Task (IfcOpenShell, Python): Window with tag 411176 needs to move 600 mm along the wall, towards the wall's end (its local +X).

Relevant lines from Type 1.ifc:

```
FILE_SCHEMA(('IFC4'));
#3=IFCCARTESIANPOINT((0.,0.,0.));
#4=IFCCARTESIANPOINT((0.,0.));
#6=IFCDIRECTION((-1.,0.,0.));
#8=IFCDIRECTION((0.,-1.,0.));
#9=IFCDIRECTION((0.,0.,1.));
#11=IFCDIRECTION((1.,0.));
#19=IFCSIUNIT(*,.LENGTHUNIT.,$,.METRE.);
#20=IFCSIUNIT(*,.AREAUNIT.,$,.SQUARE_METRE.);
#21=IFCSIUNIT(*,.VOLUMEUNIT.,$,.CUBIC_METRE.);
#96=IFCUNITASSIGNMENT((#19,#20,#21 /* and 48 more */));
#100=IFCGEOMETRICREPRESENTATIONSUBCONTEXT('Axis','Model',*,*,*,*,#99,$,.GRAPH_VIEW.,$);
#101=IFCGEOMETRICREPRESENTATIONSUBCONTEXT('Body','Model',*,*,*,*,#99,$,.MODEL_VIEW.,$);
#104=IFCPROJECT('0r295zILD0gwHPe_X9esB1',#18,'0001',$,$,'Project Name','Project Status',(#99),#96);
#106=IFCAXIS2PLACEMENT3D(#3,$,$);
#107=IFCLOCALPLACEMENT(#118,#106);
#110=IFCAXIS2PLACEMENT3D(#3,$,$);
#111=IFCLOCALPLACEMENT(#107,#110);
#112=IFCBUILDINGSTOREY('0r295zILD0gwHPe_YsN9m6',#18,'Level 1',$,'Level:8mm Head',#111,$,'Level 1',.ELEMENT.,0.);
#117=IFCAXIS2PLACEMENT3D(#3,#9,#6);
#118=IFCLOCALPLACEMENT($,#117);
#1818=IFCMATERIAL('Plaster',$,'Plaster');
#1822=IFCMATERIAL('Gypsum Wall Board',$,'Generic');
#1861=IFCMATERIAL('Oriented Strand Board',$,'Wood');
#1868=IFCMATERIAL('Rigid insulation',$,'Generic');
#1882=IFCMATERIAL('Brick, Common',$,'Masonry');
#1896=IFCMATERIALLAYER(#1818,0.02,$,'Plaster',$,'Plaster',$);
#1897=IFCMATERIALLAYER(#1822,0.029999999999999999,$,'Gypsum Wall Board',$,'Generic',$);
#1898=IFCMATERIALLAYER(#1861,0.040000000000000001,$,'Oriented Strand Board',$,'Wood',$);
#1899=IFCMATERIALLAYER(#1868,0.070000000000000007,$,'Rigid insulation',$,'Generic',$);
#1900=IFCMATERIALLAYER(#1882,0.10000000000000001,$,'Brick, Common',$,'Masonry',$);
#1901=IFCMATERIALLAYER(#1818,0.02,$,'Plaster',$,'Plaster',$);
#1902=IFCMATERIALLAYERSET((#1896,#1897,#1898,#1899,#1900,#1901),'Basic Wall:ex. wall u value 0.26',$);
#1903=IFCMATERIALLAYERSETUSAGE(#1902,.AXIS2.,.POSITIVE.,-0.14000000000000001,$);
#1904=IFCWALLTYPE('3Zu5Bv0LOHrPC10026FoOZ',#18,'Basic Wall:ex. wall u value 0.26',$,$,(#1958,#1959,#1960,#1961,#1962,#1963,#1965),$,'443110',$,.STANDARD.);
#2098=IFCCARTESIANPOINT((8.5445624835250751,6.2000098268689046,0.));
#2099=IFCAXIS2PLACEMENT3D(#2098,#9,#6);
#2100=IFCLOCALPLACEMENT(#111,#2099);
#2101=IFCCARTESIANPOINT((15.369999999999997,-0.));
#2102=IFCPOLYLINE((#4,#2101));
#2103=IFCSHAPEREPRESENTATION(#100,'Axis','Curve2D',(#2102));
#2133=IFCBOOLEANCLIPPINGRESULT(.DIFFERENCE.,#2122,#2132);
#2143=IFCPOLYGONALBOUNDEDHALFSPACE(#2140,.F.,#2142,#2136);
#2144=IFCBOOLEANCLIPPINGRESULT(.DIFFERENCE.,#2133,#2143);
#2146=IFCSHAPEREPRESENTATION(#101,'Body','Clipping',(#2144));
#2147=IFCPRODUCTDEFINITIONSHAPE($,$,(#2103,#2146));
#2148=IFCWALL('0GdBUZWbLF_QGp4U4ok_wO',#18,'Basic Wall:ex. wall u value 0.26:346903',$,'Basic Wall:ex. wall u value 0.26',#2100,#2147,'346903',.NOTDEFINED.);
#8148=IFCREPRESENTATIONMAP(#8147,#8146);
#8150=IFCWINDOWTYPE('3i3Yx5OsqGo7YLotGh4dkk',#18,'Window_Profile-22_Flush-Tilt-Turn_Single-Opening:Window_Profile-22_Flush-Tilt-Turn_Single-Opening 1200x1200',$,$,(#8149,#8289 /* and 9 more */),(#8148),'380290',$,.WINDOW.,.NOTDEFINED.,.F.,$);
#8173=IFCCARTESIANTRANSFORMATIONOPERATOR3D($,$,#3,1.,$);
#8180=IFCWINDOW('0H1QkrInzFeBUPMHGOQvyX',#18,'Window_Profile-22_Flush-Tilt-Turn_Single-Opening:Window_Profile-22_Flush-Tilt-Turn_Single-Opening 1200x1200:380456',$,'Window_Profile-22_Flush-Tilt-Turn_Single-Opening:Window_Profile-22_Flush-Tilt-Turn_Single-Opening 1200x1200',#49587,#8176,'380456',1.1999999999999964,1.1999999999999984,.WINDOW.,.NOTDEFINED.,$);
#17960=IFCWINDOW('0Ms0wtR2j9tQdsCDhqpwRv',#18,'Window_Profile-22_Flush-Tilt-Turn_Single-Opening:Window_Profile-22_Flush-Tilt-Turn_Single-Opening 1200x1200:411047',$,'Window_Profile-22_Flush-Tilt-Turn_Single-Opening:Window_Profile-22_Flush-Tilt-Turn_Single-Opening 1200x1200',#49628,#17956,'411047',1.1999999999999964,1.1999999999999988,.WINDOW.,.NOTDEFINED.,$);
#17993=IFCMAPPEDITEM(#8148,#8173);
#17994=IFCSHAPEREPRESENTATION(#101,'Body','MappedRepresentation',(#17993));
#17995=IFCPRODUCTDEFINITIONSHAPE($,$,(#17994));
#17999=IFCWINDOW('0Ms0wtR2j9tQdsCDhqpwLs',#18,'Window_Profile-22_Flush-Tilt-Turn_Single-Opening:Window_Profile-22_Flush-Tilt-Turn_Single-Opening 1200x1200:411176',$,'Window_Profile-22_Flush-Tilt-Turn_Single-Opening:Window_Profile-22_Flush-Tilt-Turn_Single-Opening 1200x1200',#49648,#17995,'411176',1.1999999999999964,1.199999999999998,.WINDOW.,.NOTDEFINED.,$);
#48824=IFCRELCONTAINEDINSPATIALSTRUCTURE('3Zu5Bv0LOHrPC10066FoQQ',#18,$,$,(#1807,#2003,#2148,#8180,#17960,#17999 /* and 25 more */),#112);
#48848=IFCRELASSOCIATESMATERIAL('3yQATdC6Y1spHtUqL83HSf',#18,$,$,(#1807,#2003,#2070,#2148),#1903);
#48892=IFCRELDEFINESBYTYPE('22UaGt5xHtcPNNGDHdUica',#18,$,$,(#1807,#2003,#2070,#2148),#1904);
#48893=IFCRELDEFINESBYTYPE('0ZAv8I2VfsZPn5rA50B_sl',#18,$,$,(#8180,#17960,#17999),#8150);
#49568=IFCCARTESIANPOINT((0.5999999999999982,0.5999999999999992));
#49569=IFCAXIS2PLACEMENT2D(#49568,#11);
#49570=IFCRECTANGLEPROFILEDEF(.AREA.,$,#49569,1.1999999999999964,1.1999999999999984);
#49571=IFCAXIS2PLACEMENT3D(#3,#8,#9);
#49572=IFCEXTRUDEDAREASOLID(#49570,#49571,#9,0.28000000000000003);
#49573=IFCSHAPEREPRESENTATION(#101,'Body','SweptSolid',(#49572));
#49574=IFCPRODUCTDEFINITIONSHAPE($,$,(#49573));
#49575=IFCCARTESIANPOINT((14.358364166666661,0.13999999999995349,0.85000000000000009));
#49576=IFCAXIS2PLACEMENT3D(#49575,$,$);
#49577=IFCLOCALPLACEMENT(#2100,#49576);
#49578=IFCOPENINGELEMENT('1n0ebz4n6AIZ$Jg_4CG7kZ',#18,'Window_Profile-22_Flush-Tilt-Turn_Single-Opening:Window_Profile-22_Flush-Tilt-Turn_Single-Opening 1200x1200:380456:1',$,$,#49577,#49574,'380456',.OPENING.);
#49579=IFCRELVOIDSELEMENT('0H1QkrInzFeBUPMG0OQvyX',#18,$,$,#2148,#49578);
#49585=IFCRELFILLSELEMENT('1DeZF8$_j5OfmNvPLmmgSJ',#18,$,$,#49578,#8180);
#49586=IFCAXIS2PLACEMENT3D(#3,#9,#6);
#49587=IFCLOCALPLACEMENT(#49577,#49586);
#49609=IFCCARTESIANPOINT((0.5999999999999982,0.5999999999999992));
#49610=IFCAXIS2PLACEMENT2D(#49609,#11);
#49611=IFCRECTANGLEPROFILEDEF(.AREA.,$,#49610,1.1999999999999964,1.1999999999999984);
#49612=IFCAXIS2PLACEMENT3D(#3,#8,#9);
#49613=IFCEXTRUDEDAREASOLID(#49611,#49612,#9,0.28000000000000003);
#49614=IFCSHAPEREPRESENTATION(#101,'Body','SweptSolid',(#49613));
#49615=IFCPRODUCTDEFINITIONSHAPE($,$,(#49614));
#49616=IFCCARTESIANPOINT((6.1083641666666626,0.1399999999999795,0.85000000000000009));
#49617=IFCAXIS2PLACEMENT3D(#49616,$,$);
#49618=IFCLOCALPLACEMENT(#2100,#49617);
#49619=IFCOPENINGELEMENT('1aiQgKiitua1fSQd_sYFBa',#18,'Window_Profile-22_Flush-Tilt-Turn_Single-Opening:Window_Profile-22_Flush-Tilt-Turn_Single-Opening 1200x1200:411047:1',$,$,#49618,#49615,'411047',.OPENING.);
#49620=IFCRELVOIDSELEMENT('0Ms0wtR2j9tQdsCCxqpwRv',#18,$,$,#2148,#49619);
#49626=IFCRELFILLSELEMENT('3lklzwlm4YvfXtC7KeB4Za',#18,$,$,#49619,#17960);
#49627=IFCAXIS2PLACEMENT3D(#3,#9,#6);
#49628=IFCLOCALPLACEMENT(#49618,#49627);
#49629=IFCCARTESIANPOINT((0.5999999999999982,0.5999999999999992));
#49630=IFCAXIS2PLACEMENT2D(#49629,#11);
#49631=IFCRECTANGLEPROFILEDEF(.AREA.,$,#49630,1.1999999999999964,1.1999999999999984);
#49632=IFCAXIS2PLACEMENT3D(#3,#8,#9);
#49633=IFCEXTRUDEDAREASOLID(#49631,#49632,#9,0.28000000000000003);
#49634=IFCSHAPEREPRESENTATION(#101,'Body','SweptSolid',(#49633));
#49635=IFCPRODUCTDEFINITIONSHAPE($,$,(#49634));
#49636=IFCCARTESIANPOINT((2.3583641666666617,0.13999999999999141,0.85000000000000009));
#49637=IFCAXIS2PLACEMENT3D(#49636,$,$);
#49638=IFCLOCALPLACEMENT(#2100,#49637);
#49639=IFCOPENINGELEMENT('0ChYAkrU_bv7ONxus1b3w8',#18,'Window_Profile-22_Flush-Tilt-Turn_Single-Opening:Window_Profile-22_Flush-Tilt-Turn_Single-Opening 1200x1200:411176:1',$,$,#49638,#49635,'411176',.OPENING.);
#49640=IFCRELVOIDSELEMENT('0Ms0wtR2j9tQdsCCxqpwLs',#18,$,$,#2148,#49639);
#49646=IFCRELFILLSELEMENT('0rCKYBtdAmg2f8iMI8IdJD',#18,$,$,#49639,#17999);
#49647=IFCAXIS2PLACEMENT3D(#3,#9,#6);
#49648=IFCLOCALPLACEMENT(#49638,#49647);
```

```python
import ifcopenshell
import ifcopenshell.api.geometry
import ifcopenshell.util.placement

model = ifcopenshell.open("Type 1.ifc")

window = model.by_id(17999)
opening = window.FillsVoids[0].RelatingOpeningElement
wall = opening.VoidsElements[0].RelatingBuildingElement

wall_matrix = ifcopenshell.util.placement.get_local_placement(wall.ObjectPlacement)
shift = wall_matrix[:3, 0] * 0.6
before = ifcopenshell.util.placement.get_local_placement(window.ObjectPlacement)[:3, 3].copy()

# The window is placed relative to its opening, so it follows when the opening moves.
matrix = ifcopenshell.util.placement.get_local_placement(opening.ObjectPlacement)
matrix[:3, 3] += shift
ifcopenshell.api.geometry.edit_object_placement(
    model, product=opening, matrix=matrix, is_si=False, should_transform_children=True
)

after = ifcopenshell.util.placement.get_local_placement(window.ObjectPlacement)[:3, 3]
print("window moved by", (after - before).round(3) + 0.0)

model.write("Type 1_updated.ifc")
```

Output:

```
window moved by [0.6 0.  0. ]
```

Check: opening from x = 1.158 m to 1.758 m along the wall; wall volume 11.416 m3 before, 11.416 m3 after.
